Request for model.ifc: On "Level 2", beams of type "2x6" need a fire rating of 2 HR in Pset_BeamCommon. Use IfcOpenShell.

First a look at what the model holds.

```python
import ifcopenshell
import ifcopenshell.util.element

model = ifcopenshell.open("model.ifc")
print(model.schema)
storey = next(s for s in model.by_type("IfcBuildingStorey") if s.Name == "Level 2")
beams = [e for e in ifcopenshell.util.element.get_decomposition(storey) if e.is_a("IfcBeam")]
seen = {}
for e in beams:
    element_type = ifcopenshell.util.element.get_type(e)
    key = (element_type.Name if element_type != e and element_type else None, ifcopenshell.util.element.get_pset(e, "Pset_BeamCommon", "FireRating"))
    seen[key] = seen.get(key, 0) + 1
for (name, value), count in sorted(seen.items(), key=str):
    print(count, "x", name, "|", value)
```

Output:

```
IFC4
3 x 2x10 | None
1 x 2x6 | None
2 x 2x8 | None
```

```python
import ifcopenshell
import ifcopenshell.api.pset
import ifcopenshell.util.element

model = ifcopenshell.open("model.ifc")

storey = next(s for s in model.by_type("IfcBuildingStorey") if s.Name == "Level 2")
beams = [e for e in ifcopenshell.util.element.get_decomposition(storey) if e.is_a("IfcBeam")]

count = 0
for e in beams:
    element_type = ifcopenshell.util.element.get_type(e)
    if element_type in (None, e) or element_type.Name != "2x6":
        continue
    # add_pset returns the element's existing set when there is one.
    pset = ifcopenshell.api.pset.add_pset(model, product=e, name="Pset_BeamCommon")
    ifcopenshell.api.pset.edit_pset(model, pset=pset, properties={"FireRating": "2 HR"})
    count += 1

print(count, "beams updated")

model.write("model_updated.ifc")
```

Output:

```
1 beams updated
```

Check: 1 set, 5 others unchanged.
